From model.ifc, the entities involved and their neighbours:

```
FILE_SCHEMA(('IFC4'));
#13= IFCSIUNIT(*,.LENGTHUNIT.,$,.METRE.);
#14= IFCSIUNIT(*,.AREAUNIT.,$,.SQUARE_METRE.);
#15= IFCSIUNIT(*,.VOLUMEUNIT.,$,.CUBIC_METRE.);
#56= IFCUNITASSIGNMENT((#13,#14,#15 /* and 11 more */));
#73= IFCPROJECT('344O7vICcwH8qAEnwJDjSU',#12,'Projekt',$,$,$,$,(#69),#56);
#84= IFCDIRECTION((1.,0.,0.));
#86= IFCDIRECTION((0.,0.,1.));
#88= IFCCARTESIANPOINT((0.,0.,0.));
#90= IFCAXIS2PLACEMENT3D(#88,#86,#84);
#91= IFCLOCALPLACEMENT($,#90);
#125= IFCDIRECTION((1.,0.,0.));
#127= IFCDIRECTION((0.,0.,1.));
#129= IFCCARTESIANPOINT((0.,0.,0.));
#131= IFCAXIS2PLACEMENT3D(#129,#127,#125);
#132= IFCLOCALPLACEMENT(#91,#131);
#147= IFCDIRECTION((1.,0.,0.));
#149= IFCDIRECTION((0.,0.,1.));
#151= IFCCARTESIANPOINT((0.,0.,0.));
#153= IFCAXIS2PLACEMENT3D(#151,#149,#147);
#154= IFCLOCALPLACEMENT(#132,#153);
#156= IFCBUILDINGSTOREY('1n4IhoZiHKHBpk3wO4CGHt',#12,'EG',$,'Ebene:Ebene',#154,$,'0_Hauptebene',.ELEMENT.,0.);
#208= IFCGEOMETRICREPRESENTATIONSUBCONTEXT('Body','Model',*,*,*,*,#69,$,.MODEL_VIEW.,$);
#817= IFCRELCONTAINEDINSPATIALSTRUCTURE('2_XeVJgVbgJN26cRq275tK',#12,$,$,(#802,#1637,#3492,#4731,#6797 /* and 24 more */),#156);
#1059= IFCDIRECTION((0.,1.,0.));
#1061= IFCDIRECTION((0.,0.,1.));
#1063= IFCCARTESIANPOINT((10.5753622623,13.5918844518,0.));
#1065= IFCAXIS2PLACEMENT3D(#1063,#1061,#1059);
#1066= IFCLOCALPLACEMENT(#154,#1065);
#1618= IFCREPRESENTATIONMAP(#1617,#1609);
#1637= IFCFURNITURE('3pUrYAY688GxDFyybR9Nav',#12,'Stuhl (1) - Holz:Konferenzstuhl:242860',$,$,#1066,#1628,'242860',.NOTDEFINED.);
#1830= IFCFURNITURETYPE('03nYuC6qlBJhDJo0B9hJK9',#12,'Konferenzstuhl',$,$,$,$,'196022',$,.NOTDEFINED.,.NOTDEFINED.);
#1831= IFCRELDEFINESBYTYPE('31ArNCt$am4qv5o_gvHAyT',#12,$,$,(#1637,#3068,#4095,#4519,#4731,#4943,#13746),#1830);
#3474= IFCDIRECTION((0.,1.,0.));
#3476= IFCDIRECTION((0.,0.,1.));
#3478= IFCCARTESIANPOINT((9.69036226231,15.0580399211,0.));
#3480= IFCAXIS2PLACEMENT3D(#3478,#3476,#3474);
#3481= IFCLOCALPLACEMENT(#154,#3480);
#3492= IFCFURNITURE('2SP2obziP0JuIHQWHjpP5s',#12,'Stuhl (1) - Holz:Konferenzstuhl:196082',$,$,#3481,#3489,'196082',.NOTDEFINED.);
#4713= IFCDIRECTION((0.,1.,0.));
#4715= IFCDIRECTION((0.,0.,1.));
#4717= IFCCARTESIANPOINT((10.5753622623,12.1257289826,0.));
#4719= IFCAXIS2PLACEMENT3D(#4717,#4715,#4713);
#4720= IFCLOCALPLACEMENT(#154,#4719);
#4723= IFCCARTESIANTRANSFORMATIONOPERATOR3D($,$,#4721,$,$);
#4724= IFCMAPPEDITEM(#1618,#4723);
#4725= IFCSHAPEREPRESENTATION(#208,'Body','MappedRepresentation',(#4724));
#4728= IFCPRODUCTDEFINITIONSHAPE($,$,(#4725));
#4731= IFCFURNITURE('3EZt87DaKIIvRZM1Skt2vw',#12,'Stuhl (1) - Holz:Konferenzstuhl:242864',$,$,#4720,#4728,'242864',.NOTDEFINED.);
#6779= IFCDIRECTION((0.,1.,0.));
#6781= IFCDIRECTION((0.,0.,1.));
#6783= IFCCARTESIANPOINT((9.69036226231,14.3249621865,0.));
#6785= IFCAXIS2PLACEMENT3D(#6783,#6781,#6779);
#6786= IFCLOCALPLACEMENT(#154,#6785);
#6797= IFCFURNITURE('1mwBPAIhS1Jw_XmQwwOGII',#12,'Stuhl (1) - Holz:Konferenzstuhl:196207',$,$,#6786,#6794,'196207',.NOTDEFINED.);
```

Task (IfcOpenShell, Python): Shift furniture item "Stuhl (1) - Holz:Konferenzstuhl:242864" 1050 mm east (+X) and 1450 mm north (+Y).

```python
import ifcopenshell
import ifcopenshell.api.geometry
import ifcopenshell.util.placement
import ifcopenshell.util.unit

model = ifcopenshell.open("model.ifc")
unit_scale = ifcopenshell.util.unit.calculate_unit_scale(model)

item = model.by_id(4731)
matrix = ifcopenshell.util.placement.get_local_placement(item.ObjectPlacement)
matrix[0, 3] += 1.05 / unit_scale
matrix[1, 3] += 1.45 / unit_scale
ifcopenshell.api.geometry.edit_object_placement(model, product=item, matrix=matrix, is_si=False)

print(ifcopenshell.util.placement.get_local_placement(item.ObjectPlacement).round(3) + 0.0)

model.write("model_rev.ifc")
```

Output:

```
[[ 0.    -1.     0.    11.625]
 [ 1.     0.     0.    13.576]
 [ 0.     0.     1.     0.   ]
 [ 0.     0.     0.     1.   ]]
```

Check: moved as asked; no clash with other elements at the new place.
